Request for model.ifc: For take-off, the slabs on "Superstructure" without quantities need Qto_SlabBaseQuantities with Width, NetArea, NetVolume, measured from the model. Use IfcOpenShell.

First a look at what the model holds.

```python
import ifcopenshell
import ifcopenshell.util.element
import ifcopenshell.util.unit

model = ifcopenshell.open("model.ifc")
print(model.schema)
for unit_type in ("LENGTHUNIT", "AREAUNIT", "VOLUMEUNIT"):
    print(unit_type, ifcopenshell.util.unit.calculate_unit_scale(model, unit_type))
storey = next(s for s in model.by_type("IfcBuildingStorey") if s.Name == "Superstructure")
slabs = [e for e in ifcopenshell.util.element.get_decomposition(storey) if e.is_a("IfcSlab")]
for e in sorted(slabs, key=lambda e: e.id()):
    print(e.id(), e.is_a(), e.Name, list(ifcopenshell.util.element.get_psets(e, qtos_only=True)), sep=" | ")
```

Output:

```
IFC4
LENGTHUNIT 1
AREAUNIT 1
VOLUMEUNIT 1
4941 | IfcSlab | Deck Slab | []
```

```python
import ifcopenshell
import ifcopenshell.api.pset
import ifcopenshell.geom
import ifcopenshell.util.element
import ifcopenshell.util.shape
import ifcopenshell.util.unit

model = ifcopenshell.open("model.ifc")
unit_scale = ifcopenshell.util.unit.calculate_unit_scale(model)
area_scale = ifcopenshell.util.unit.calculate_unit_scale(model, "AREAUNIT")
volume_scale = ifcopenshell.util.unit.calculate_unit_scale(model, "VOLUMEUNIT")
settings = ifcopenshell.geom.settings()

storey = next(s for s in model.by_type("IfcBuildingStorey") if s.Name == "Superstructure")
slabs = [e for e in ifcopenshell.util.element.get_decomposition(storey) if e.is_a("IfcSlab")]

for e in sorted(slabs, key=lambda e: e.id()):
    if ifcopenshell.util.element.get_psets(e, qtos_only=True, should_inherit=False):
        continue
    # Geometry comes back in metres, in the element's own axes.
    shape = ifcopenshell.geom.create_shape(settings, e)
    values = {
        "Width": ifcopenshell.util.shape.get_z(shape.geometry) / unit_scale,
        "NetArea": ifcopenshell.util.shape.get_footprint_area(shape.geometry) / area_scale,
        "NetVolume": ifcopenshell.util.shape.get_volume(shape.geometry) / volume_scale,
    }
    qto = ifcopenshell.api.pset.add_qto(model, product=e, name="Qto_SlabBaseQuantities")
    ifcopenshell.api.pset.edit_qto(model, qto=qto, properties=values)
    print(e.id(), {k: round(v, 3) for k, v in values.items()})

model.write("model_rev.ifc")
```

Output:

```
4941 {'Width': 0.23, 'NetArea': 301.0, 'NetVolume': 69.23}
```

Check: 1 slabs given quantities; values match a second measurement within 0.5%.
